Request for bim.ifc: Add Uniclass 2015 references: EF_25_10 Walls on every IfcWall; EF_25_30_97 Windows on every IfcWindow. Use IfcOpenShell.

First a look at what the model holds.

```python
import ifcopenshell

model = ifcopenshell.open("bim.ifc")
print(model.schema)
print("classifications:", [c.Name for c in model.by_type("IfcClassification")])
for ifc_class in ("IfcDoor", "IfcRoof", "IfcStair", "IfcWall", "IfcWindow"):
    print(ifc_class, len(model.by_type(ifc_class)))
```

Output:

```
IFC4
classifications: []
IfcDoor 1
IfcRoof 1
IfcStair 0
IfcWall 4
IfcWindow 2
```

```python
import ifcopenshell
import ifcopenshell.api.classification

model = ifcopenshell.open("bim.ifc")

system = ifcopenshell.api.classification.add_classification(model, classification="Uniclass 2015")

codes = {
    "IfcWall": ("EF_25_10", "Walls"),
    "IfcWindow": ("EF_25_30_97", "Windows"),
}
for ifc_class, (code, name) in codes.items():
    products = model.by_type(ifc_class)
    ifcopenshell.api.classification.add_reference(
        model, products=products, classification=system, identification=code, name=name
    )
    print(code, len(products))

model.write("bim_v2.ifc")
```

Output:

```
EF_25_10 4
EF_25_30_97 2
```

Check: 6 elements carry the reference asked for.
